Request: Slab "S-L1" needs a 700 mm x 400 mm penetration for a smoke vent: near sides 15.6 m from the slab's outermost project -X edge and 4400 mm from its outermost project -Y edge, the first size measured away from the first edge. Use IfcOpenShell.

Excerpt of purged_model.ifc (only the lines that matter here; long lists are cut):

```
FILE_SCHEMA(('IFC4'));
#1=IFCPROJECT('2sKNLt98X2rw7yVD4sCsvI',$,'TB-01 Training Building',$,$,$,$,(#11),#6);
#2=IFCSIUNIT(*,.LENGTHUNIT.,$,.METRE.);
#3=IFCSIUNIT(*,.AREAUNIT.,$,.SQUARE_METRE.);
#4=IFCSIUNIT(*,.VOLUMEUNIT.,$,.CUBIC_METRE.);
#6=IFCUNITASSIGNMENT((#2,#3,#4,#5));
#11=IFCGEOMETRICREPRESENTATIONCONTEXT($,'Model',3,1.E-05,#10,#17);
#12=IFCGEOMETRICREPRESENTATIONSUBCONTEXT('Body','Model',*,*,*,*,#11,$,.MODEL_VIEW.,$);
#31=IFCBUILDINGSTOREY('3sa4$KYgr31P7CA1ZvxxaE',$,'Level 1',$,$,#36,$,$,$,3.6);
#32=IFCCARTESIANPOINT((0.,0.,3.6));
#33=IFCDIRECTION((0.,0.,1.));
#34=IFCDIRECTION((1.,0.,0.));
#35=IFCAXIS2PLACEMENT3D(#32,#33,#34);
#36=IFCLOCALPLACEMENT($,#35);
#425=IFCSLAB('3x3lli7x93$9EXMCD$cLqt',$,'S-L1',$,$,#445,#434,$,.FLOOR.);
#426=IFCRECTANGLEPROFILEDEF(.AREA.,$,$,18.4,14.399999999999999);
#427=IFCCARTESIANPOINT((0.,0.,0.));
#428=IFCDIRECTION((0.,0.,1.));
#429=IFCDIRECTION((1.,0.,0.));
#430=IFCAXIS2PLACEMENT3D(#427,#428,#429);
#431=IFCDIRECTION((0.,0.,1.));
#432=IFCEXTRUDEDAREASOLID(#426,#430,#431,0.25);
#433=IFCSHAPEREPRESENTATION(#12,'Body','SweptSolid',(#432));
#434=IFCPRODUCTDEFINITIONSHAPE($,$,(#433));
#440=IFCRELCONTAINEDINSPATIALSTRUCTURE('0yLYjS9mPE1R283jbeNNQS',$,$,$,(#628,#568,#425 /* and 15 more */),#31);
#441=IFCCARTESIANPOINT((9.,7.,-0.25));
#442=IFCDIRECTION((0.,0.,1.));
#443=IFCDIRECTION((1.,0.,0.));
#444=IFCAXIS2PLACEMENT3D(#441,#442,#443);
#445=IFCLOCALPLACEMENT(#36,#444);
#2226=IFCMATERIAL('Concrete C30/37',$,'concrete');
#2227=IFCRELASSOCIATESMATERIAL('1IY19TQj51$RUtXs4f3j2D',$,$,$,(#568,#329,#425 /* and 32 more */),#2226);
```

```python
import numpy as np
import ifcopenshell
import ifcopenshell.api.feature
import ifcopenshell.api.geometry
import ifcopenshell.api.root
import ifcopenshell.geom
import ifcopenshell.util.placement
import ifcopenshell.util.representation
import ifcopenshell.util.shape
import ifcopenshell.util.unit

model = ifcopenshell.open("purged_model.ifc")
unit_scale = ifcopenshell.util.unit.calculate_unit_scale(model)
settings = ifcopenshell.geom.settings()


def volume(element):
    """Net volume in cubic metres, openings subtracted."""
    shape = ifcopenshell.geom.create_shape(settings, element)
    return ifcopenshell.util.shape.get_volume(shape.geometry)


slab = model.by_guid("3x3lli7x93$9EXMCD$cLqt")
before = volume(slab)

# Extent in the slab's own axes, in metres. The edges named are its -X and -Y sides.
slab_shape = ifcopenshell.geom.create_shape(settings, slab)
vertices = ifcopenshell.util.shape.get_vertices(slab_shape.geometry)
x_min, y_min, bottom = vertices.min(axis=0)
top = vertices[:, 2].max()

opening = ifcopenshell.api.root.create_entity(model, ifc_class="IfcOpeningElement", name="Smoke vent opening", predefined_type="OPENING")
context = ifcopenshell.util.representation.get_context(model, "Model", "Body", "MODEL_VIEW")
width, depth = 0.7, 0.4
outline = [(0.0, 0.0), (width, 0.0), (width, depth), (0.0, depth), (0.0, 0.0)]
# Overshoot both faces by 50 mm so the cut is clean.
shape = ifcopenshell.api.geometry.add_slab_representation(
    model, context=context, depth=top - bottom + 0.1, polyline=outline
)
ifcopenshell.api.geometry.assign_representation(model, product=opening, representation=shape)

matrix = ifcopenshell.util.placement.get_local_placement(slab.ObjectPlacement)
matrix[:, 3] = matrix @ np.append(np.array([x_min + 15.6, y_min + 4.4, bottom - 0.05]) / unit_scale, 1.0)
ifcopenshell.api.geometry.edit_object_placement(model, product=opening, matrix=matrix, is_si=False)
ifcopenshell.api.feature.add_feature(model, feature=opening, element=slab)

after = volume(slab)

print(f"slab volume {before:.3f} -> {after:.3f} m3")

model.write("purged_model_v2.ifc")
```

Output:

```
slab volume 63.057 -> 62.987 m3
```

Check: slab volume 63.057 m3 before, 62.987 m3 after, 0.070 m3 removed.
